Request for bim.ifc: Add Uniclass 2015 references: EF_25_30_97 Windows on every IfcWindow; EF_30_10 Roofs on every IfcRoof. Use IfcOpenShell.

First a look at what the model holds.

```python
import ifcopenshell

model = ifcopenshell.open("bim.ifc")
print(model.schema)
print("classifications:", [c.Name for c in model.by_type("IfcClassification")])
for ifc_class in ("IfcDoor", "IfcRoof", "IfcStair", "IfcWall", "IfcWindow"):
    print(ifc_class, len(model.by_type(ifc_class)))
```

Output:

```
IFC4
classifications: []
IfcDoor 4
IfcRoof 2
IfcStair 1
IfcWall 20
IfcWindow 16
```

```python
import ifcopenshell
import ifcopenshell.api.classification

model = ifcopenshell.open("bim.ifc")

system = ifcopenshell.api.classification.add_classification(model, classification="Uniclass 2015")

codes = {
    "IfcWindow": ("EF_25_30_97", "Windows"),
    "IfcRoof": ("EF_30_10", "Roofs"),
}
for ifc_class, (code, name) in codes.items():
    products = model.by_type(ifc_class)
    ifcopenshell.api.classification.add_reference(
        model, products=products, classification=system, identification=code, name=name
    )
    print(code, len(products))

model.write("bim_updated.ifc")
```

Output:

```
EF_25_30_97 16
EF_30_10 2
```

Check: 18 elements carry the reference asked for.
